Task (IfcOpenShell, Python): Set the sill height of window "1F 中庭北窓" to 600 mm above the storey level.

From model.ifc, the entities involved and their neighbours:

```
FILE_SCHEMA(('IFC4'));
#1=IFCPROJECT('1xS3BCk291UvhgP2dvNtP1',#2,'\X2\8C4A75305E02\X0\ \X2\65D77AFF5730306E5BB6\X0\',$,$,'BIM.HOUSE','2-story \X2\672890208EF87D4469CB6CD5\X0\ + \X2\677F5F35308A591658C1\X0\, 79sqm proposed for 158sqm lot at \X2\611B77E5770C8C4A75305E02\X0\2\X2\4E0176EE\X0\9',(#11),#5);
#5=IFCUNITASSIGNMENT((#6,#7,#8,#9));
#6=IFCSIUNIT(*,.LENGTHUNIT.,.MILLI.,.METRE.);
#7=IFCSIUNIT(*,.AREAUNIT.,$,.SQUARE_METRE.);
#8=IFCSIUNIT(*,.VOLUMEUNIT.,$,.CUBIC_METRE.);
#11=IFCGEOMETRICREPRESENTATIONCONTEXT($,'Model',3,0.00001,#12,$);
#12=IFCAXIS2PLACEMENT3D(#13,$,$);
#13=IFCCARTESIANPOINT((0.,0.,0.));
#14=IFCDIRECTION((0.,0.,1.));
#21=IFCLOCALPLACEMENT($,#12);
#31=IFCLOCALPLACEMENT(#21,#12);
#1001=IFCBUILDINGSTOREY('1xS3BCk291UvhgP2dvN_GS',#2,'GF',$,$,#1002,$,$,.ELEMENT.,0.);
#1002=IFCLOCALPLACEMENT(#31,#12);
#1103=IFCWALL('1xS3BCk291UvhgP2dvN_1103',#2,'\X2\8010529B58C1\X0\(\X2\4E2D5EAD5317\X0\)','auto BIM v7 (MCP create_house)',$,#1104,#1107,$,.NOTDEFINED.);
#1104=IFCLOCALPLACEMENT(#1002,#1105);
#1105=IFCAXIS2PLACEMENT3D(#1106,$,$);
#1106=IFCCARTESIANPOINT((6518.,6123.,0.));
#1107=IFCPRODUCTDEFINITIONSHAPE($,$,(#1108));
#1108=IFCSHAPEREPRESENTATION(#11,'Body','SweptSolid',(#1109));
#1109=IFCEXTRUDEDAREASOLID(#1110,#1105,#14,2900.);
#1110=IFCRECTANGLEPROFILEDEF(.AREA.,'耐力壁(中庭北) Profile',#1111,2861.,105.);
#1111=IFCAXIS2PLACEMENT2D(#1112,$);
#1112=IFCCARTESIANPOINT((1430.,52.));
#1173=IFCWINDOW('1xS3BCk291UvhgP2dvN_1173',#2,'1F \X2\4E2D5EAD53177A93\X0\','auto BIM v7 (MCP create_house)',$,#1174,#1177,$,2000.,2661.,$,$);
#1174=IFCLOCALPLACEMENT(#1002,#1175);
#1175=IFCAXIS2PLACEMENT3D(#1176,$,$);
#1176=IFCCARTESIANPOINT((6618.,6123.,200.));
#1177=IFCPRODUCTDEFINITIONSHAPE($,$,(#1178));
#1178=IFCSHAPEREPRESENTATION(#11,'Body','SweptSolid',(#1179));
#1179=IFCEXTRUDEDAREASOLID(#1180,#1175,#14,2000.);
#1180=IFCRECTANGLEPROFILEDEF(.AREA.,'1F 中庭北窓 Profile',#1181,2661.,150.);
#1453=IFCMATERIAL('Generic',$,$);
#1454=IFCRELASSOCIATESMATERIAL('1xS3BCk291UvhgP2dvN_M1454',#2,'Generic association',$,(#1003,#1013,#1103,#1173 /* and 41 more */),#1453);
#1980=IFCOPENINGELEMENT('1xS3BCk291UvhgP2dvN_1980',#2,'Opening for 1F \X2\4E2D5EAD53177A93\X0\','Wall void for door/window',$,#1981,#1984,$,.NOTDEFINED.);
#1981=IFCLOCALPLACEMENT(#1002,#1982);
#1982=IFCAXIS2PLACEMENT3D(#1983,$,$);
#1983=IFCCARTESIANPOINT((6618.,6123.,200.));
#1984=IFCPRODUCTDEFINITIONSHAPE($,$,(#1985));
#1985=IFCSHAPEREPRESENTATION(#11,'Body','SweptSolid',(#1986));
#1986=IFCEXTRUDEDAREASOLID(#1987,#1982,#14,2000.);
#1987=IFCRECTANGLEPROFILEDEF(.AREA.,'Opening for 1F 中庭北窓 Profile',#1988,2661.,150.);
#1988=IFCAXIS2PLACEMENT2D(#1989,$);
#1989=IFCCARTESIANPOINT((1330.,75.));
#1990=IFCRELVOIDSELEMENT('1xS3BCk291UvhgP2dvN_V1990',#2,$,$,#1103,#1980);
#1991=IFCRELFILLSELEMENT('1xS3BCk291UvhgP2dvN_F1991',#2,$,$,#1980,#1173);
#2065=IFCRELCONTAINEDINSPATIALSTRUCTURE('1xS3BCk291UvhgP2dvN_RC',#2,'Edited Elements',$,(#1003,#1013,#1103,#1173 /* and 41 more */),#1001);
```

```python
import numpy as np
import ifcopenshell
import ifcopenshell.api.geometry
import ifcopenshell.geom
import ifcopenshell.util.element
import ifcopenshell.util.placement
import ifcopenshell.util.shape
import ifcopenshell.util.unit

model = ifcopenshell.open("model.ifc")
unit_scale = ifcopenshell.util.unit.calculate_unit_scale(model)

window = model.by_id(1173)
opening = window.FillsVoids[0].RelatingOpeningElement
storey = ifcopenshell.util.element.get_container(window, ifc_class="IfcBuildingStorey")
level = ifcopenshell.util.placement.get_local_placement(storey.ObjectPlacement)[2, 3]

# The opening's origin need not be at the sill, so measure its lowest point.
shape = ifcopenshell.geom.create_shape(ifcopenshell.geom.settings(), opening)
bottom = ifcopenshell.util.shape.get_shape_bottom_elevation(shape, shape.geometry) / unit_scale
dz = level + 600.0 - bottom

shift = np.array([0.0, 0.0, dz])
# The window is not placed relative to its opening, so move both.
for product in (opening, window):
    matrix = ifcopenshell.util.placement.get_local_placement(product.ObjectPlacement)
    matrix[:3, 3] += shift
    ifcopenshell.api.geometry.edit_object_placement(model, product=product, matrix=matrix, is_si=False)

print(f"moved by {dz * unit_scale:+.3f} m")

model.write("model_updated.ifc")
```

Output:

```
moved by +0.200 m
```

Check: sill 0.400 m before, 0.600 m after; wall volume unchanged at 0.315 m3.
